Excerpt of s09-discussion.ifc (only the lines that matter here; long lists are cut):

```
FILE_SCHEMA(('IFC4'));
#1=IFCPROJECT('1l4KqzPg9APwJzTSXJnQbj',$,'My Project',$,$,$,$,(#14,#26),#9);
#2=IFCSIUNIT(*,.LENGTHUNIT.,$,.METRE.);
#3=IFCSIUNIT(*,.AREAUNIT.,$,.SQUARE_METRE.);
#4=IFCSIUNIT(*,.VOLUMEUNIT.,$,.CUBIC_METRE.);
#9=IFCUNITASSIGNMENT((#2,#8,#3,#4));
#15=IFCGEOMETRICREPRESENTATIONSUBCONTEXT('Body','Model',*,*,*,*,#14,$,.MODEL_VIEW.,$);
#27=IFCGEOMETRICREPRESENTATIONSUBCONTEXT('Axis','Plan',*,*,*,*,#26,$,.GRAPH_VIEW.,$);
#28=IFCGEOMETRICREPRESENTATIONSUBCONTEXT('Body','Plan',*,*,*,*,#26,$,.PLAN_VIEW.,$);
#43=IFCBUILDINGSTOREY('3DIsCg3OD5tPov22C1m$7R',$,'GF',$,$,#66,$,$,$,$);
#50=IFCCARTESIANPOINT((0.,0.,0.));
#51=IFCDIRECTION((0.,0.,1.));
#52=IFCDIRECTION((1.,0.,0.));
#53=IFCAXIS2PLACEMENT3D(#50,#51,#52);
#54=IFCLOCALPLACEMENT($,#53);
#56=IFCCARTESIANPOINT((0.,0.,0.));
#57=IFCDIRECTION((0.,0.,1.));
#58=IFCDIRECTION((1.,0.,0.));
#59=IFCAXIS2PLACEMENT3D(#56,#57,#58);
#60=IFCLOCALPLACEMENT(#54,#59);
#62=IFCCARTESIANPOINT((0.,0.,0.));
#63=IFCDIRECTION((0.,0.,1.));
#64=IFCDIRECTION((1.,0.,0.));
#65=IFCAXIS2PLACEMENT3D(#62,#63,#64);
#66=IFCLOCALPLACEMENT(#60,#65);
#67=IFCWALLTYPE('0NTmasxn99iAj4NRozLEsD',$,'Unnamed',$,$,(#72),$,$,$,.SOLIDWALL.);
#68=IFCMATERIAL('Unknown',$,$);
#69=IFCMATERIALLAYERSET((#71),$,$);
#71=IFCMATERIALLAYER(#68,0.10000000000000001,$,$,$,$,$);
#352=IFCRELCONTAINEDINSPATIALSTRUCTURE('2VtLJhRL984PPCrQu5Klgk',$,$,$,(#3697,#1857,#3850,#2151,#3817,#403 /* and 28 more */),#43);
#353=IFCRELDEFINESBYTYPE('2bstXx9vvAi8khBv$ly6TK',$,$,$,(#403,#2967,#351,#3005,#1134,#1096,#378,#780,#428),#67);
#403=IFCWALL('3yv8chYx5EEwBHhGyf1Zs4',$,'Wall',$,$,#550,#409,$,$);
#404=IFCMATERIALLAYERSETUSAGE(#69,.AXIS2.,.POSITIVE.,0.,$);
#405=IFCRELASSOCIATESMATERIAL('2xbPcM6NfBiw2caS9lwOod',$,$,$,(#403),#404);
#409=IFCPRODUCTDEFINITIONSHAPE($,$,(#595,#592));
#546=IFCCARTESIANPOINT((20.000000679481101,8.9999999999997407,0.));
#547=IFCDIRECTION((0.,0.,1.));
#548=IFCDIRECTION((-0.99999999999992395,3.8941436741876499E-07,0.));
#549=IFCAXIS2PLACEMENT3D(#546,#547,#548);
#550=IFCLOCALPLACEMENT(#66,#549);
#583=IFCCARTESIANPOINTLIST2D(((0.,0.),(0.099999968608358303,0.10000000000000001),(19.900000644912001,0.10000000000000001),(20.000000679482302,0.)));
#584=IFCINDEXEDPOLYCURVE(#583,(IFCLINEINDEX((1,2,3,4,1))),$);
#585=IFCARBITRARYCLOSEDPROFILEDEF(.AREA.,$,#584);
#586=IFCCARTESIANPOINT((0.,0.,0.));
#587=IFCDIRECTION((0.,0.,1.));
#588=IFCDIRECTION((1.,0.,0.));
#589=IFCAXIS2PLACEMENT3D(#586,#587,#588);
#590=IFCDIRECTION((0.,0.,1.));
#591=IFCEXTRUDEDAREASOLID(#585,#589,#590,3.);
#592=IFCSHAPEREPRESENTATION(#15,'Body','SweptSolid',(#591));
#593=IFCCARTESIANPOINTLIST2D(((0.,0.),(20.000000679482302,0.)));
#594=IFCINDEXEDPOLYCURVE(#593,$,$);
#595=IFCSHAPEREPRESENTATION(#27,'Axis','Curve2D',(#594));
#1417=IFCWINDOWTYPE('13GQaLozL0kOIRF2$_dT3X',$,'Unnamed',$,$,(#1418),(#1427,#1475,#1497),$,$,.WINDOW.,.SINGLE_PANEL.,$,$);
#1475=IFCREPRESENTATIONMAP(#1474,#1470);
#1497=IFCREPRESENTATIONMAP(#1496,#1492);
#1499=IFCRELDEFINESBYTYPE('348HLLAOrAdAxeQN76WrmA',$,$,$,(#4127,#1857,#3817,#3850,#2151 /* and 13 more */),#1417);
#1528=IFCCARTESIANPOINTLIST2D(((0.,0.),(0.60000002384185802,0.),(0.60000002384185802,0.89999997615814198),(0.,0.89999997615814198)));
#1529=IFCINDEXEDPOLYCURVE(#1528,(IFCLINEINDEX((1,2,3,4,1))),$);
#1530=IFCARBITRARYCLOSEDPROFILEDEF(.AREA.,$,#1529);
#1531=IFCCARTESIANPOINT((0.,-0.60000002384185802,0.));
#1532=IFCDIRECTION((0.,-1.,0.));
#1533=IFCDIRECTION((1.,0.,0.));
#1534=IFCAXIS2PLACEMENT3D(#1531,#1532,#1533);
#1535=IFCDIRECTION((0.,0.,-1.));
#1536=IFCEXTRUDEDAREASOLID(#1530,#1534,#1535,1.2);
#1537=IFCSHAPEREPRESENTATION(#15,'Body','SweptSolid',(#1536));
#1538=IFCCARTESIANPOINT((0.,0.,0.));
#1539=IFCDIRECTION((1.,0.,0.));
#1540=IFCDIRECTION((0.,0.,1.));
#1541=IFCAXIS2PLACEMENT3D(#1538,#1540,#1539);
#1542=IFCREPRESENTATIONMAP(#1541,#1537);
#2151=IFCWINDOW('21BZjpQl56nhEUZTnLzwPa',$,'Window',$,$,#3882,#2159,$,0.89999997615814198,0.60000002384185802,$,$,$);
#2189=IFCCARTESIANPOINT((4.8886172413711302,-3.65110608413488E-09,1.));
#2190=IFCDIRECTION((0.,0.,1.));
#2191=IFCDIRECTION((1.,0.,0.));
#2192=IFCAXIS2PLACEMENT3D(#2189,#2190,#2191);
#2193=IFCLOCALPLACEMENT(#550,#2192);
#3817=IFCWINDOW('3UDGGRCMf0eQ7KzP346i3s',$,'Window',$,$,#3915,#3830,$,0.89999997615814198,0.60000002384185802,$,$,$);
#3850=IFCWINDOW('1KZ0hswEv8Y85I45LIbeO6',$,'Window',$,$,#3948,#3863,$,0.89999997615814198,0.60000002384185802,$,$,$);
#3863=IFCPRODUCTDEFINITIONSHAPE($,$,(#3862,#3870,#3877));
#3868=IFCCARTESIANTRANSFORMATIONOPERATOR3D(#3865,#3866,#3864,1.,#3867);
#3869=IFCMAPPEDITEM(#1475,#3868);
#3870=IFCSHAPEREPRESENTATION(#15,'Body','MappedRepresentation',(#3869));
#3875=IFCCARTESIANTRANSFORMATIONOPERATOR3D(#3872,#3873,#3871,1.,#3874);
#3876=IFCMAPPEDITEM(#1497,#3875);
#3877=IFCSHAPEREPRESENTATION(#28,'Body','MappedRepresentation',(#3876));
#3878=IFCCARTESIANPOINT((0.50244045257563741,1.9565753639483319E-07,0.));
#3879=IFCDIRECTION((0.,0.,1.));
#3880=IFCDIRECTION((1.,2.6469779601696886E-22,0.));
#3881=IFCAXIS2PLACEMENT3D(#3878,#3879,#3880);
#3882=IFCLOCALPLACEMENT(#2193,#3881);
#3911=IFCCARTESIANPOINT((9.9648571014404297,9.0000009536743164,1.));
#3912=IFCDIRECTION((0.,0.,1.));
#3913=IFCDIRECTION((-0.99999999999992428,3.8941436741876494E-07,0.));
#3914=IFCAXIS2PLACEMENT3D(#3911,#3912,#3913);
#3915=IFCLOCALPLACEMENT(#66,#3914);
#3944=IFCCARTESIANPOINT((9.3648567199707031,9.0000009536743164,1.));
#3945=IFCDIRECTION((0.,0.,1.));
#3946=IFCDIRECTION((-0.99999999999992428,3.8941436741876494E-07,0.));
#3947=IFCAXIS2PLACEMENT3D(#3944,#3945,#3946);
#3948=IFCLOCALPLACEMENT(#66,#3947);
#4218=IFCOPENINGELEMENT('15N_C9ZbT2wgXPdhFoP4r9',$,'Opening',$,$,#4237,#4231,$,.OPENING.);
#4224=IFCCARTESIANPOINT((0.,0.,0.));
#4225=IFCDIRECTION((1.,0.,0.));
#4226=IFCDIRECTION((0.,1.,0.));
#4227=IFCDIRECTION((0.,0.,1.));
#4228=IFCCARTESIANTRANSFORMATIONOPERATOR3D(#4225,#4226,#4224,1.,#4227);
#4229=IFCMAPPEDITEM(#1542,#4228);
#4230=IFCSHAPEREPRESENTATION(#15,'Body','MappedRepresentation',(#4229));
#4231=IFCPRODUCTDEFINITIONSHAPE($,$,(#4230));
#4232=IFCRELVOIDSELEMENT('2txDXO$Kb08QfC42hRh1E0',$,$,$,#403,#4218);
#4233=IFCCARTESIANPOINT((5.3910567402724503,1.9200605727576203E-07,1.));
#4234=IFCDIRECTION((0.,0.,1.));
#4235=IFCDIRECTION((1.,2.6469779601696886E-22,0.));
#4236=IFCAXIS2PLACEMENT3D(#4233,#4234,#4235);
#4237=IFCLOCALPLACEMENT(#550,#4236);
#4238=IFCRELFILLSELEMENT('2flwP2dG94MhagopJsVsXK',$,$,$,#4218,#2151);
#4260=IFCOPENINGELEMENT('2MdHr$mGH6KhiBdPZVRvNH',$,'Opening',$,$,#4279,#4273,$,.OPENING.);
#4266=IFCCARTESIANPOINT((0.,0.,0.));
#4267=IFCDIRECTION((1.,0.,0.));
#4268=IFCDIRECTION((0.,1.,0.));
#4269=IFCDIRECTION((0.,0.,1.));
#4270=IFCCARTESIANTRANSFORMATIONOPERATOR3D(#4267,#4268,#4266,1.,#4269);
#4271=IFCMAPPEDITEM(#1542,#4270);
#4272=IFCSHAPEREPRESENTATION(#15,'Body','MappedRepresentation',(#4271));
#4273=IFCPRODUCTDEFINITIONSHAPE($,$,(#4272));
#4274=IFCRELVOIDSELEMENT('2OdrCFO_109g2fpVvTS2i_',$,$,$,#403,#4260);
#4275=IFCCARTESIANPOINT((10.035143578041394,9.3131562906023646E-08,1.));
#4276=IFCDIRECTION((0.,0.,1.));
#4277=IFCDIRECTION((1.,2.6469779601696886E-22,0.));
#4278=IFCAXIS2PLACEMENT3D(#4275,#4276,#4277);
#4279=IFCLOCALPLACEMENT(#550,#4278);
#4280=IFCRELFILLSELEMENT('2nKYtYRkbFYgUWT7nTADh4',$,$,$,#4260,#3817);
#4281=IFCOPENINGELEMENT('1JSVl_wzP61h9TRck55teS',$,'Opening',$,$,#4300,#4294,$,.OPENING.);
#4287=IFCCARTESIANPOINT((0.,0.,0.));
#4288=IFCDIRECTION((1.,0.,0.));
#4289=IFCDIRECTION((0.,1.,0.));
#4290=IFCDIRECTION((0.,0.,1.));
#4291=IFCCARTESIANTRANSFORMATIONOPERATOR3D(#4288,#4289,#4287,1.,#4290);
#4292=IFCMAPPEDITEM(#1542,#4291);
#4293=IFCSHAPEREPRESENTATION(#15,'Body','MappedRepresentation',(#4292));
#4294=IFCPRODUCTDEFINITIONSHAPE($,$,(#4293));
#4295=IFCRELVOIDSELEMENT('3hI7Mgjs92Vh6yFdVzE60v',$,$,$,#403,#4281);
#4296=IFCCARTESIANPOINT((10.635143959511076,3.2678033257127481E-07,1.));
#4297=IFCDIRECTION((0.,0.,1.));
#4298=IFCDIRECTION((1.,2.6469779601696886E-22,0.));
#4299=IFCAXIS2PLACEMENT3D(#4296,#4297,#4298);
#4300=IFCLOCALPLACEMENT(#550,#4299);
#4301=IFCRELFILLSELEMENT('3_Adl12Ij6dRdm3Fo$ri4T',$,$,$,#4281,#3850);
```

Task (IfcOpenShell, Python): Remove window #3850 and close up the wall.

```python
import ifcopenshell
import ifcopenshell.api.feature
import ifcopenshell.api.root
import ifcopenshell.geom
import ifcopenshell.util.shape

model = ifcopenshell.open("s09-discussion.ifc")
settings = ifcopenshell.geom.settings()


def volume(element):
    """Net volume in cubic metres, openings subtracted."""
    shape = ifcopenshell.geom.create_shape(settings, element)
    return ifcopenshell.util.shape.get_volume(shape.geometry)


window = model.by_guid("1KZ0hswEv8Y85I45LIbeO6")
opening = window.FillsVoids[0].RelatingOpeningElement
wall = opening.VoidsElements[0].RelatingBuildingElement
before = volume(wall)

ifcopenshell.api.root.remove_product(model, product=window)
ifcopenshell.api.feature.remove_feature(model, feature=opening)

after = volume(wall)

print(f"wall volume {before:.3f} -> {after:.3f} m3")

model.write("s09-discussion_rev.ifc")
```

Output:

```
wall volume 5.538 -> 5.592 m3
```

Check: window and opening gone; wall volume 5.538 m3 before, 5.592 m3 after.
